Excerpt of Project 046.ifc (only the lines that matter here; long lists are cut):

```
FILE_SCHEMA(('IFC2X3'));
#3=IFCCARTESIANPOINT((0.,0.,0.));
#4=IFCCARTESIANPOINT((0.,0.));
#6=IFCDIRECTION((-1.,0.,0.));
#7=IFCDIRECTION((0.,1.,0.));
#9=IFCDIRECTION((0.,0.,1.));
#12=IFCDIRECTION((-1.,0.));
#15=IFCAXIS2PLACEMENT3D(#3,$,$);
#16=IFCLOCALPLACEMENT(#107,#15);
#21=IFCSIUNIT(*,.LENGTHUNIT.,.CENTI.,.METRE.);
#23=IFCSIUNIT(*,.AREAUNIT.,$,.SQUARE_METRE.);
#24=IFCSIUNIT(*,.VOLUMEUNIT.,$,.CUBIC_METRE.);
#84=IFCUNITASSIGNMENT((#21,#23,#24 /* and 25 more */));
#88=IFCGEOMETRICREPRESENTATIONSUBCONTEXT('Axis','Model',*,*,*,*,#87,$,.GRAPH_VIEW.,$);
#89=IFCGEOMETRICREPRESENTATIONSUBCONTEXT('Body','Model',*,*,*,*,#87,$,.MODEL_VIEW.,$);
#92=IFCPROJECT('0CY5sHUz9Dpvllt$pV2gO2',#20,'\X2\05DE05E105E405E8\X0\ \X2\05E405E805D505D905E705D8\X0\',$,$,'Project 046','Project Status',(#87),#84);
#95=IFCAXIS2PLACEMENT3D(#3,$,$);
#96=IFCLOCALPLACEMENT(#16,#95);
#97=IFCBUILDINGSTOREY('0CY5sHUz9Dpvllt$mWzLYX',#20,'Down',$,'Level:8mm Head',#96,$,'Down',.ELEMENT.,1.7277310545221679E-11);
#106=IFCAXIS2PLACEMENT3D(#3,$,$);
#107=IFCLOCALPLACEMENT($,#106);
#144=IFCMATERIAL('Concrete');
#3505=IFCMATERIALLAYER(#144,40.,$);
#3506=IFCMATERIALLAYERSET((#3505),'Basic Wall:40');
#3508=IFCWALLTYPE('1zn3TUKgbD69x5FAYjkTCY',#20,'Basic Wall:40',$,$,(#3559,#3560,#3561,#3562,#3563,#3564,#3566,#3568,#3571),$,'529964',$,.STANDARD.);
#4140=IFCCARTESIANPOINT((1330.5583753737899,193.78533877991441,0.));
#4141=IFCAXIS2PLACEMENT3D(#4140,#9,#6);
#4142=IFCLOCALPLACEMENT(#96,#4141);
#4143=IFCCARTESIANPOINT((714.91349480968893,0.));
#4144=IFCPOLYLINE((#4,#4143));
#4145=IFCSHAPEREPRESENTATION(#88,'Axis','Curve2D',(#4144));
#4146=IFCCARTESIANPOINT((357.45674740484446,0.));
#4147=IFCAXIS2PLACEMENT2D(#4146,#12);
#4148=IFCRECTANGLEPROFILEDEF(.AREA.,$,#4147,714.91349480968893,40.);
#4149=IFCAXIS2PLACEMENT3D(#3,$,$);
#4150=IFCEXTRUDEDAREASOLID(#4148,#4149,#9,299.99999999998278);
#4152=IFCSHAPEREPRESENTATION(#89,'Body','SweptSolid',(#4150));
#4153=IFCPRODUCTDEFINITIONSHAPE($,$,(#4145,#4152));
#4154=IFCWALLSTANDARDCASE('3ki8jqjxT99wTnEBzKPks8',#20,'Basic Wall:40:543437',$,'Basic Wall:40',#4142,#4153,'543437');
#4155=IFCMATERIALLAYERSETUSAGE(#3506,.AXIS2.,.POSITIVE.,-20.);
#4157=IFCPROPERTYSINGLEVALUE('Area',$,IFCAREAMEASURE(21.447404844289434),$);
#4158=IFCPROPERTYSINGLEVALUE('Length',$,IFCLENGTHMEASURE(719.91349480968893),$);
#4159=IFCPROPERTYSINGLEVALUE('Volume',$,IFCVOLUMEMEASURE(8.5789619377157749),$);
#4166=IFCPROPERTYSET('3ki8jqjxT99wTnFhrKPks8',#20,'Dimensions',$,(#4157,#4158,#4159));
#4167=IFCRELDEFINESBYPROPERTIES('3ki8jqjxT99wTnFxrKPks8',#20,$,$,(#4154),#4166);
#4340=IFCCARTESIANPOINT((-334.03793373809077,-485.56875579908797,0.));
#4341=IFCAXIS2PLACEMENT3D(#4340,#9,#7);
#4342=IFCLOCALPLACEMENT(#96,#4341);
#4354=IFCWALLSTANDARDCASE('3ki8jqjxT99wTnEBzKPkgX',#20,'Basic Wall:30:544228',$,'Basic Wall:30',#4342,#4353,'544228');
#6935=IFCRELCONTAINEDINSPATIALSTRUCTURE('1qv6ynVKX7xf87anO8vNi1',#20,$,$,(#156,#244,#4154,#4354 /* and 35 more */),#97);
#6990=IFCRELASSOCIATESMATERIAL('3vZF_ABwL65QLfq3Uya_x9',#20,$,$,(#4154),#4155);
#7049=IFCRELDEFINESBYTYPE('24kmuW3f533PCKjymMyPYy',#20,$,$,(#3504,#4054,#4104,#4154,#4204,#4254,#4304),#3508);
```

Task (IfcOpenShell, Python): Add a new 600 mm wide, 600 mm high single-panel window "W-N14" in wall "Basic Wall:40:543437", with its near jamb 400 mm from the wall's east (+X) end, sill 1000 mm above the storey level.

```python
import numpy as np
import ifcopenshell
import ifcopenshell.api.feature
import ifcopenshell.api.geometry
import ifcopenshell.api.pset
import ifcopenshell.api.root
import ifcopenshell.api.spatial
import ifcopenshell.api.type
import ifcopenshell.geom
import ifcopenshell.util.element
import ifcopenshell.util.placement
import ifcopenshell.util.representation
import ifcopenshell.util.shape
import ifcopenshell.util.unit

model = ifcopenshell.open("Project 046.ifc")
unit_scale = ifcopenshell.util.unit.calculate_unit_scale(model)
area_scale = ifcopenshell.util.unit.calculate_unit_scale(model, "AREAUNIT")
volume_scale = ifcopenshell.util.unit.calculate_unit_scale(model, "VOLUMEUNIT")
settings = ifcopenshell.geom.settings()


def volume(element):
    """Net volume in cubic metres, openings subtracted."""
    shape = ifcopenshell.geom.create_shape(settings, element)
    return ifcopenshell.util.shape.get_volume(shape.geometry)


wall = model.by_guid("3ki8jqjxT99wTnEBzKPks8")
storey = ifcopenshell.util.element.get_container(wall, ifc_class="IfcBuildingStorey")
context = ifcopenshell.util.representation.get_context(model, "Model", "Body", "MODEL_VIEW")
before = volume(wall)

width, height, from_end, sill = 0.6, 0.6, 0.4, 1  # metres

# The wall runs along its own X axis, and the end named is its -X end.
wall_shape = ifcopenshell.geom.create_shape(settings, wall)
x, y, z = ifcopenshell.util.shape.get_vertices(wall_shape.geometry).T
start = x.min() + from_end
face, thickness = float(y.min()), float(y.max() - y.min())
wall_matrix = ifcopenshell.util.placement.get_local_placement(wall.ObjectPlacement)
level = ifcopenshell.util.placement.get_local_placement(storey.ObjectPlacement)[2, 3]


def in_wall(x, y):
    """Placement at x, y metres in the wall's axes, at sill height."""
    matrix = wall_matrix.copy()
    matrix[:, 3] = wall_matrix @ np.array([x / unit_scale, y / unit_scale, 0.0, 1.0])
    matrix[2, 3] = level + sill / unit_scale
    return matrix


# Opening: a box that overshoots both wall faces by 50 mm.
opening = ifcopenshell.api.root.create_entity(model, ifc_class="IfcOpeningElement")
box = ifcopenshell.api.geometry.add_wall_representation(
    model, context=context, length=width, height=height, thickness=thickness + 0.1
)
ifcopenshell.api.geometry.assign_representation(model, product=opening, representation=box)
ifcopenshell.api.geometry.edit_object_placement(model, product=opening, matrix=in_wall(start, face - 0.05), is_si=False)
ifcopenshell.api.feature.add_feature(model, feature=opening, element=wall)

window = ifcopenshell.api.root.create_entity(model, ifc_class="IfcWindow", name="W-N14")
window.OverallWidth, window.OverallHeight = width / unit_scale, height / unit_scale
body = ifcopenshell.api.geometry.add_window_representation(
    model,
    context=context,
    overall_width=window.OverallWidth,
    overall_height=window.OverallHeight,
    partition_type="SINGLE_PANEL",
)
ifcopenshell.api.geometry.assign_representation(model, product=window, representation=body)
ifcopenshell.api.spatial.assign_container(model, products=[window], relating_structure=storey)
fills = ifcopenshell.api.feature.add_filling(model, opening=opening, element=window)
fills.OwnerHistory = window.OwnerHistory  # required in IFC2X3

# IFC2X3 keeps the operation on the window style.
style = ifcopenshell.api.root.create_entity(model, ifc_class="IfcWindowStyle", name="W-N14")
style.OperationType, style.ConstructionType = "SINGLE_PANEL", "NOTDEFINED"
style.ParameterTakesPrecedence = style.Sizeable = False
ifcopenshell.api.type.assign_type(model, related_objects=[window], relating_type=style)

# Centre the window in the wall's thickness.
ifcopenshell.api.geometry.edit_object_placement(model, product=window, matrix=in_wall(start, face), is_si=False)
window_shape = ifcopenshell.geom.create_shape(settings, window)
depth = ifcopenshell.util.shape.get_vertices(window_shape.geometry)[:, 1]
offset = face + thickness / 2 - (depth.min() + depth.max()) / 2
ifcopenshell.api.geometry.edit_object_placement(model, product=window, matrix=in_wall(start, offset), is_si=False)

after = volume(wall)

# Update the wall's stored quantities.
pset = model.by_id(ifcopenshell.util.element.get_pset(wall, "Dimensions", should_inherit=False)["id"])
ifcopenshell.api.pset.edit_pset(model, pset=pset, properties={
    "Area": model.create_entity("IfcAreaMeasure", after / thickness / area_scale),
    "Volume": model.create_entity("IfcVolumeMeasure", after / volume_scale),
})

print(f"wall volume {before:.3f} -> {after:.3f} m3")

model.write("Project 046-out.ifc")
```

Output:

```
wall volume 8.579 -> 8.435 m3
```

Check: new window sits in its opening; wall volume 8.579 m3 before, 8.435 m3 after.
